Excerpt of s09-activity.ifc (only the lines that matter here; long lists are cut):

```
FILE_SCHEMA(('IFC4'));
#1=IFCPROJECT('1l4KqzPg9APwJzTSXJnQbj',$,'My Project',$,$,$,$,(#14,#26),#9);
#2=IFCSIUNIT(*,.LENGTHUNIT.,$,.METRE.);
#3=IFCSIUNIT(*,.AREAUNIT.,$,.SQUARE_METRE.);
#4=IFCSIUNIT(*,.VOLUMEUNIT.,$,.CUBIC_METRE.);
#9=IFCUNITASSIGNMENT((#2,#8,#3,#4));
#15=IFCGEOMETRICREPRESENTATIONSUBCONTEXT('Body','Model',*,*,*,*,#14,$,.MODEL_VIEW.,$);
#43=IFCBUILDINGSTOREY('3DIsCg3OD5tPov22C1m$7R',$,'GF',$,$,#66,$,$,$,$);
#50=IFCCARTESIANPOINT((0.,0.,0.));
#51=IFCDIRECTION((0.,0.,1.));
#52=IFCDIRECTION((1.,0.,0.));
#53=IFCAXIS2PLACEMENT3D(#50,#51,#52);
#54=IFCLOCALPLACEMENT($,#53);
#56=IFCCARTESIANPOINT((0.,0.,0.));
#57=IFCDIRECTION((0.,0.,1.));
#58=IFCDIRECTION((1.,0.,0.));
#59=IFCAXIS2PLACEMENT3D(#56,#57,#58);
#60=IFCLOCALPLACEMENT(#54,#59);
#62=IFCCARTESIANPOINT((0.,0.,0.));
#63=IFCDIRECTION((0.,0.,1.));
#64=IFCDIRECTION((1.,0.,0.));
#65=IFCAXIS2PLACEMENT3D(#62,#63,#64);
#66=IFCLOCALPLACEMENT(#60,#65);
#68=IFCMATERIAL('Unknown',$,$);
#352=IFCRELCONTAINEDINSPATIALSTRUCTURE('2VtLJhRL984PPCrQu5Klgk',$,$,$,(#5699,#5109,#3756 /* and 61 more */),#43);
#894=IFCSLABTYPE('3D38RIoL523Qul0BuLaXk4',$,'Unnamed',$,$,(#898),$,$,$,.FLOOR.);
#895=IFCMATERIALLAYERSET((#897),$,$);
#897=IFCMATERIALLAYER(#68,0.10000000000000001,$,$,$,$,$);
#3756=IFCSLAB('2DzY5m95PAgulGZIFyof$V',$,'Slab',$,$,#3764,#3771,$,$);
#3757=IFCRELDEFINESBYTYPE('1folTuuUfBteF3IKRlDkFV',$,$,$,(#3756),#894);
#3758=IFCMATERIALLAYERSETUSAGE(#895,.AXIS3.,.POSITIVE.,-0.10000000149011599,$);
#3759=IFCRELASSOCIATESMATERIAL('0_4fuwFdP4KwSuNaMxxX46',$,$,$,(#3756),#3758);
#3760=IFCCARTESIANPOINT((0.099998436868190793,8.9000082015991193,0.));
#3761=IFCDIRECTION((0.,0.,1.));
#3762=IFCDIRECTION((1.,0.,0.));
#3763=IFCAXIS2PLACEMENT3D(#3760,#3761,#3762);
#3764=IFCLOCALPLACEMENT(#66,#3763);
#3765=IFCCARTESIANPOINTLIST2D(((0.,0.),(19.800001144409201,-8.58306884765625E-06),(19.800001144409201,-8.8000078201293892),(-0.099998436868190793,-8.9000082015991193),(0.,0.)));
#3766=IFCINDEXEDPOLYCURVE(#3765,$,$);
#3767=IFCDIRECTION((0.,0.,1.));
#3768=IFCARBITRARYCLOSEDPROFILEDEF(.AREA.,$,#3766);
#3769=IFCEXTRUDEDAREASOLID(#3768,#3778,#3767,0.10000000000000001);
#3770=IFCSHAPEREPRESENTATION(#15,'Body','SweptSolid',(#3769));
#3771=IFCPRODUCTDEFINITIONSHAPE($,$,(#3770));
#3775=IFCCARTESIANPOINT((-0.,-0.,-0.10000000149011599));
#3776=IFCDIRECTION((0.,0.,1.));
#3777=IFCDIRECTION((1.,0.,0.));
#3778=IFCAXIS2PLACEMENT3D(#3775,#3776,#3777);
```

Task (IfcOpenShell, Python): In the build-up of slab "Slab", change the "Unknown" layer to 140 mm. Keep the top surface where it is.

```python
import ifcopenshell
import ifcopenshell.util.element
import ifcopenshell.util.representation

model = ifcopenshell.open("s09-activity.ifc")

layer_set = model.by_id(895)
layer = next(l for l in layer_set.MaterialLayers if l.Material and l.Material.Name == "Unknown")
change = 0.14 - layer.LayerThickness
layer.LayerThickness += change

# Geometry does not follow the layer set by itself.
slabs = [e for e in ifcopenshell.util.element.get_elements_by_material(model, layer_set) if e.is_a("IfcSlab")]
for slab in sorted(slabs, key=lambda e: e.id()):
    body = ifcopenshell.util.representation.get_representation(slab, "Model", "Body")
    solid = body.Items[0]
    old_depth = solid.Depth
    solid.Depth += change
    # Extruded upwards: lower the start of the extrusion so the top stays.
    x, y, z = solid.Position.Location.Coordinates
    solid.Position.Location = model.createIfcCartesianPoint((x, y, z - change))
    print(slab.id(), f"{old_depth:g} -> {solid.Depth:g}")

# The layers are counted up from the underside, which has moved.
for usage in {ifcopenshell.util.element.get_material(slab) for slab in slabs}:
    usage.OffsetFromReferenceLine -= change

model.write("s09-activity_edited.ifc")
```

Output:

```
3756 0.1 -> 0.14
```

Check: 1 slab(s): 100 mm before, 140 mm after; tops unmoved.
